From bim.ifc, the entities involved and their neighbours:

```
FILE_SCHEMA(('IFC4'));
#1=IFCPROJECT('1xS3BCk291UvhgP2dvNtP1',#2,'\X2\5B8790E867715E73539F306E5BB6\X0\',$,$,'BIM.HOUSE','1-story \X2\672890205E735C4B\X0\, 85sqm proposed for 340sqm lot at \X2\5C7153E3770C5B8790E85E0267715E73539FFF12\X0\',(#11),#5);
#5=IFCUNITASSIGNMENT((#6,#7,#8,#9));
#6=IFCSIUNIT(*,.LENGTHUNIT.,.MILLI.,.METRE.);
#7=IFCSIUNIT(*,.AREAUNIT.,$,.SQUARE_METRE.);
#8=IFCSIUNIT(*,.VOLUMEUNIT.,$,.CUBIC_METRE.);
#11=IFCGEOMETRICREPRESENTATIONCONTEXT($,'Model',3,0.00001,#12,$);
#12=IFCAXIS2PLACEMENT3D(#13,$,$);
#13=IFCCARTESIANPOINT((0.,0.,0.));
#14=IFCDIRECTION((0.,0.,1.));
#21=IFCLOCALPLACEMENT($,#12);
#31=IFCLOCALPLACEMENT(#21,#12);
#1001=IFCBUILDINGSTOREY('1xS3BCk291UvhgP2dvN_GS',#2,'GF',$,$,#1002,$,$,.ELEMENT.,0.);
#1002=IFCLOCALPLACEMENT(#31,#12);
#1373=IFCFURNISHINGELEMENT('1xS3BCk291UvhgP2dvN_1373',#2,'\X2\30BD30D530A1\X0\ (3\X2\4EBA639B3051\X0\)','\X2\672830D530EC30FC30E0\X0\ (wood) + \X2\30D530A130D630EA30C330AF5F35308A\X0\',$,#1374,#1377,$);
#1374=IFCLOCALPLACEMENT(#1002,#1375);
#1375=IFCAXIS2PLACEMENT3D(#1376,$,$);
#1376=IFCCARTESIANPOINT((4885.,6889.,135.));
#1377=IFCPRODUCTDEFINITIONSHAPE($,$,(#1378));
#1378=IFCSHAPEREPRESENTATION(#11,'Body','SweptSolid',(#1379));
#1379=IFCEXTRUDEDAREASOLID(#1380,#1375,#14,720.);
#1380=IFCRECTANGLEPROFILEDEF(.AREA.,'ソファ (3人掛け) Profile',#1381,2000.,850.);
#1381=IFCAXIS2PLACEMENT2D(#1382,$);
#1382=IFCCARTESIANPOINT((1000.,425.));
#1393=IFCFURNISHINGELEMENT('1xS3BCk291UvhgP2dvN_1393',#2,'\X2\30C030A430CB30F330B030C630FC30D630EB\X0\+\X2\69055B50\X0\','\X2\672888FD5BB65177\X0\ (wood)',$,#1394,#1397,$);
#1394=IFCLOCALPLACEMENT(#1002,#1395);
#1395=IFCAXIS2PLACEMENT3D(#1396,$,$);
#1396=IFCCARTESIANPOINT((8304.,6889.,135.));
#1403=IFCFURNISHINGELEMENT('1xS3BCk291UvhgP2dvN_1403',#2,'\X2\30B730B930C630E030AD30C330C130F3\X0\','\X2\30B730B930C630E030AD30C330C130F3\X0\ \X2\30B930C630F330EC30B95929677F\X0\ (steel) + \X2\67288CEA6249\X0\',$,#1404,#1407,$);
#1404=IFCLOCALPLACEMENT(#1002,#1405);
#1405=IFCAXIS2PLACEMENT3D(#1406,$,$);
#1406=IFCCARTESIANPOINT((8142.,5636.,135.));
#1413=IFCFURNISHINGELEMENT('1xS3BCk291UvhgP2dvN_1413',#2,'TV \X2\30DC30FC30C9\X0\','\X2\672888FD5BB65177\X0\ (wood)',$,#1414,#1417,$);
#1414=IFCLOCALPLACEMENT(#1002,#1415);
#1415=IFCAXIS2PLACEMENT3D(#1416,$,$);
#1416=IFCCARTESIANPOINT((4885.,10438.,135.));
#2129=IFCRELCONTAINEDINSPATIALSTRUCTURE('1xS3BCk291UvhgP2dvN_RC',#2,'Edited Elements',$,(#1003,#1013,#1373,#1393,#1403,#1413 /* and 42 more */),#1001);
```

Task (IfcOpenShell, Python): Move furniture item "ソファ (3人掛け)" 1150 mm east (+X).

```python
import ifcopenshell
import ifcopenshell.api.geometry
import ifcopenshell.util.placement

model = ifcopenshell.open("bim.ifc")

item = model.by_guid("1xS3BCk291UvhgP2dvN_1373")
matrix = ifcopenshell.util.placement.get_local_placement(item.ObjectPlacement)
matrix[0, 3] += 1150.0
ifcopenshell.api.geometry.edit_object_placement(model, product=item, matrix=matrix, is_si=False)

print(ifcopenshell.util.placement.get_local_placement(item.ObjectPlacement).round(3) + 0.0)

model.write("bim_edited.ifc")
```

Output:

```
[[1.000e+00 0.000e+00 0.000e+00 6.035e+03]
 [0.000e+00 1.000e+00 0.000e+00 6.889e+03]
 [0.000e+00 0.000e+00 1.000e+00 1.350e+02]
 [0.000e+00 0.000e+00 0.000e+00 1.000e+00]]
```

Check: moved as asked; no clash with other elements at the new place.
